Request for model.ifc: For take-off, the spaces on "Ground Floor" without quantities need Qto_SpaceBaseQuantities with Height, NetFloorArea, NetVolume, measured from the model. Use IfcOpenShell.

First a look at what the model holds.

```python
import ifcopenshell
import ifcopenshell.util.element
import ifcopenshell.util.unit

model = ifcopenshell.open("model.ifc")
print(model.schema)
for unit_type in ("LENGTHUNIT", "AREAUNIT", "VOLUMEUNIT"):
    print(unit_type, ifcopenshell.util.unit.calculate_unit_scale(model, unit_type))
storey = next(s for s in model.by_type("IfcBuildingStorey") if s.Name == "Ground Floor")
spaces = [e for e in ifcopenshell.util.element.get_decomposition(storey) if e.is_a("IfcSpace")]
for e in sorted(spaces, key=lambda e: e.id()):
    print(e.id(), e.is_a(), e.Name, list(ifcopenshell.util.element.get_psets(e, qtos_only=True)), sep=" | ")
```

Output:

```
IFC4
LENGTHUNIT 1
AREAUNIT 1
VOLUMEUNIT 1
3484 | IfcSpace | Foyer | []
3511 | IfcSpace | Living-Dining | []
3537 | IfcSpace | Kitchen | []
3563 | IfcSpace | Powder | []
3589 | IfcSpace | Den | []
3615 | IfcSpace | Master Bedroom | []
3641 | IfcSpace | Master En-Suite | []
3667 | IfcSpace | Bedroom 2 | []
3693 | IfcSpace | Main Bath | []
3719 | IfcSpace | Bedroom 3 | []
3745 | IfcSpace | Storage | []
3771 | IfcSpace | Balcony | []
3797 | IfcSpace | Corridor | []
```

```python
import ifcopenshell
import ifcopenshell.api.pset
import ifcopenshell.geom
import ifcopenshell.util.element
import ifcopenshell.util.shape
import ifcopenshell.util.unit

model = ifcopenshell.open("model.ifc")
unit_scale = ifcopenshell.util.unit.calculate_unit_scale(model)
area_scale = ifcopenshell.util.unit.calculate_unit_scale(model, "AREAUNIT")
volume_scale = ifcopenshell.util.unit.calculate_unit_scale(model, "VOLUMEUNIT")
settings = ifcopenshell.geom.settings()

storey = next(s for s in model.by_type("IfcBuildingStorey") if s.Name == "Ground Floor")
spaces = [e for e in ifcopenshell.util.element.get_decomposition(storey) if e.is_a("IfcSpace")]

for e in sorted(spaces, key=lambda e: e.id()):
    if ifcopenshell.util.element.get_psets(e, qtos_only=True, should_inherit=False):
        continue
    # Geometry comes back in metres, in the element's own axes.
    shape = ifcopenshell.geom.create_shape(settings, e)
    values = {
        "Height": ifcopenshell.util.shape.get_z(shape.geometry) / unit_scale,
        "NetFloorArea": ifcopenshell.util.shape.get_footprint_area(shape.geometry) / area_scale,
        "NetVolume": ifcopenshell.util.shape.get_volume(shape.geometry) / volume_scale,
    }
    qto = ifcopenshell.api.pset.add_qto(model, product=e, name="Qto_SpaceBaseQuantities")
    ifcopenshell.api.pset.edit_qto(model, qto=qto, properties=values)
    print(e.id(), {k: round(v, 3) for k, v in values.items()})

model.write("model_edited.ifc")
```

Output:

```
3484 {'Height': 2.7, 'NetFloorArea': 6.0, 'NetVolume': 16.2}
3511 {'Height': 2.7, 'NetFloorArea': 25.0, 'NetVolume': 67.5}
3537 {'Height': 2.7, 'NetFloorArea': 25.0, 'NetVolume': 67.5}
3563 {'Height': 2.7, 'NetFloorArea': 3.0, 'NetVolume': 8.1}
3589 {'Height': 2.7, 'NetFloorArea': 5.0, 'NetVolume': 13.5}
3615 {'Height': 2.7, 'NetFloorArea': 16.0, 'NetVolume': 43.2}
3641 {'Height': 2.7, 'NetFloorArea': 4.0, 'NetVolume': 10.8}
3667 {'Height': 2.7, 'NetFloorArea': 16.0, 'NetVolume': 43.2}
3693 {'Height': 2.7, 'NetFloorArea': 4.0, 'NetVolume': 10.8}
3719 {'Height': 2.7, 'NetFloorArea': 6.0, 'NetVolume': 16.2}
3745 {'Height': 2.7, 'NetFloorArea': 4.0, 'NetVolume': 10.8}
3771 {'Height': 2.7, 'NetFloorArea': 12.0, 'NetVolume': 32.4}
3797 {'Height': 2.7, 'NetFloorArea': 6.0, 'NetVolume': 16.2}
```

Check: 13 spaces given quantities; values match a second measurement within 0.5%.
